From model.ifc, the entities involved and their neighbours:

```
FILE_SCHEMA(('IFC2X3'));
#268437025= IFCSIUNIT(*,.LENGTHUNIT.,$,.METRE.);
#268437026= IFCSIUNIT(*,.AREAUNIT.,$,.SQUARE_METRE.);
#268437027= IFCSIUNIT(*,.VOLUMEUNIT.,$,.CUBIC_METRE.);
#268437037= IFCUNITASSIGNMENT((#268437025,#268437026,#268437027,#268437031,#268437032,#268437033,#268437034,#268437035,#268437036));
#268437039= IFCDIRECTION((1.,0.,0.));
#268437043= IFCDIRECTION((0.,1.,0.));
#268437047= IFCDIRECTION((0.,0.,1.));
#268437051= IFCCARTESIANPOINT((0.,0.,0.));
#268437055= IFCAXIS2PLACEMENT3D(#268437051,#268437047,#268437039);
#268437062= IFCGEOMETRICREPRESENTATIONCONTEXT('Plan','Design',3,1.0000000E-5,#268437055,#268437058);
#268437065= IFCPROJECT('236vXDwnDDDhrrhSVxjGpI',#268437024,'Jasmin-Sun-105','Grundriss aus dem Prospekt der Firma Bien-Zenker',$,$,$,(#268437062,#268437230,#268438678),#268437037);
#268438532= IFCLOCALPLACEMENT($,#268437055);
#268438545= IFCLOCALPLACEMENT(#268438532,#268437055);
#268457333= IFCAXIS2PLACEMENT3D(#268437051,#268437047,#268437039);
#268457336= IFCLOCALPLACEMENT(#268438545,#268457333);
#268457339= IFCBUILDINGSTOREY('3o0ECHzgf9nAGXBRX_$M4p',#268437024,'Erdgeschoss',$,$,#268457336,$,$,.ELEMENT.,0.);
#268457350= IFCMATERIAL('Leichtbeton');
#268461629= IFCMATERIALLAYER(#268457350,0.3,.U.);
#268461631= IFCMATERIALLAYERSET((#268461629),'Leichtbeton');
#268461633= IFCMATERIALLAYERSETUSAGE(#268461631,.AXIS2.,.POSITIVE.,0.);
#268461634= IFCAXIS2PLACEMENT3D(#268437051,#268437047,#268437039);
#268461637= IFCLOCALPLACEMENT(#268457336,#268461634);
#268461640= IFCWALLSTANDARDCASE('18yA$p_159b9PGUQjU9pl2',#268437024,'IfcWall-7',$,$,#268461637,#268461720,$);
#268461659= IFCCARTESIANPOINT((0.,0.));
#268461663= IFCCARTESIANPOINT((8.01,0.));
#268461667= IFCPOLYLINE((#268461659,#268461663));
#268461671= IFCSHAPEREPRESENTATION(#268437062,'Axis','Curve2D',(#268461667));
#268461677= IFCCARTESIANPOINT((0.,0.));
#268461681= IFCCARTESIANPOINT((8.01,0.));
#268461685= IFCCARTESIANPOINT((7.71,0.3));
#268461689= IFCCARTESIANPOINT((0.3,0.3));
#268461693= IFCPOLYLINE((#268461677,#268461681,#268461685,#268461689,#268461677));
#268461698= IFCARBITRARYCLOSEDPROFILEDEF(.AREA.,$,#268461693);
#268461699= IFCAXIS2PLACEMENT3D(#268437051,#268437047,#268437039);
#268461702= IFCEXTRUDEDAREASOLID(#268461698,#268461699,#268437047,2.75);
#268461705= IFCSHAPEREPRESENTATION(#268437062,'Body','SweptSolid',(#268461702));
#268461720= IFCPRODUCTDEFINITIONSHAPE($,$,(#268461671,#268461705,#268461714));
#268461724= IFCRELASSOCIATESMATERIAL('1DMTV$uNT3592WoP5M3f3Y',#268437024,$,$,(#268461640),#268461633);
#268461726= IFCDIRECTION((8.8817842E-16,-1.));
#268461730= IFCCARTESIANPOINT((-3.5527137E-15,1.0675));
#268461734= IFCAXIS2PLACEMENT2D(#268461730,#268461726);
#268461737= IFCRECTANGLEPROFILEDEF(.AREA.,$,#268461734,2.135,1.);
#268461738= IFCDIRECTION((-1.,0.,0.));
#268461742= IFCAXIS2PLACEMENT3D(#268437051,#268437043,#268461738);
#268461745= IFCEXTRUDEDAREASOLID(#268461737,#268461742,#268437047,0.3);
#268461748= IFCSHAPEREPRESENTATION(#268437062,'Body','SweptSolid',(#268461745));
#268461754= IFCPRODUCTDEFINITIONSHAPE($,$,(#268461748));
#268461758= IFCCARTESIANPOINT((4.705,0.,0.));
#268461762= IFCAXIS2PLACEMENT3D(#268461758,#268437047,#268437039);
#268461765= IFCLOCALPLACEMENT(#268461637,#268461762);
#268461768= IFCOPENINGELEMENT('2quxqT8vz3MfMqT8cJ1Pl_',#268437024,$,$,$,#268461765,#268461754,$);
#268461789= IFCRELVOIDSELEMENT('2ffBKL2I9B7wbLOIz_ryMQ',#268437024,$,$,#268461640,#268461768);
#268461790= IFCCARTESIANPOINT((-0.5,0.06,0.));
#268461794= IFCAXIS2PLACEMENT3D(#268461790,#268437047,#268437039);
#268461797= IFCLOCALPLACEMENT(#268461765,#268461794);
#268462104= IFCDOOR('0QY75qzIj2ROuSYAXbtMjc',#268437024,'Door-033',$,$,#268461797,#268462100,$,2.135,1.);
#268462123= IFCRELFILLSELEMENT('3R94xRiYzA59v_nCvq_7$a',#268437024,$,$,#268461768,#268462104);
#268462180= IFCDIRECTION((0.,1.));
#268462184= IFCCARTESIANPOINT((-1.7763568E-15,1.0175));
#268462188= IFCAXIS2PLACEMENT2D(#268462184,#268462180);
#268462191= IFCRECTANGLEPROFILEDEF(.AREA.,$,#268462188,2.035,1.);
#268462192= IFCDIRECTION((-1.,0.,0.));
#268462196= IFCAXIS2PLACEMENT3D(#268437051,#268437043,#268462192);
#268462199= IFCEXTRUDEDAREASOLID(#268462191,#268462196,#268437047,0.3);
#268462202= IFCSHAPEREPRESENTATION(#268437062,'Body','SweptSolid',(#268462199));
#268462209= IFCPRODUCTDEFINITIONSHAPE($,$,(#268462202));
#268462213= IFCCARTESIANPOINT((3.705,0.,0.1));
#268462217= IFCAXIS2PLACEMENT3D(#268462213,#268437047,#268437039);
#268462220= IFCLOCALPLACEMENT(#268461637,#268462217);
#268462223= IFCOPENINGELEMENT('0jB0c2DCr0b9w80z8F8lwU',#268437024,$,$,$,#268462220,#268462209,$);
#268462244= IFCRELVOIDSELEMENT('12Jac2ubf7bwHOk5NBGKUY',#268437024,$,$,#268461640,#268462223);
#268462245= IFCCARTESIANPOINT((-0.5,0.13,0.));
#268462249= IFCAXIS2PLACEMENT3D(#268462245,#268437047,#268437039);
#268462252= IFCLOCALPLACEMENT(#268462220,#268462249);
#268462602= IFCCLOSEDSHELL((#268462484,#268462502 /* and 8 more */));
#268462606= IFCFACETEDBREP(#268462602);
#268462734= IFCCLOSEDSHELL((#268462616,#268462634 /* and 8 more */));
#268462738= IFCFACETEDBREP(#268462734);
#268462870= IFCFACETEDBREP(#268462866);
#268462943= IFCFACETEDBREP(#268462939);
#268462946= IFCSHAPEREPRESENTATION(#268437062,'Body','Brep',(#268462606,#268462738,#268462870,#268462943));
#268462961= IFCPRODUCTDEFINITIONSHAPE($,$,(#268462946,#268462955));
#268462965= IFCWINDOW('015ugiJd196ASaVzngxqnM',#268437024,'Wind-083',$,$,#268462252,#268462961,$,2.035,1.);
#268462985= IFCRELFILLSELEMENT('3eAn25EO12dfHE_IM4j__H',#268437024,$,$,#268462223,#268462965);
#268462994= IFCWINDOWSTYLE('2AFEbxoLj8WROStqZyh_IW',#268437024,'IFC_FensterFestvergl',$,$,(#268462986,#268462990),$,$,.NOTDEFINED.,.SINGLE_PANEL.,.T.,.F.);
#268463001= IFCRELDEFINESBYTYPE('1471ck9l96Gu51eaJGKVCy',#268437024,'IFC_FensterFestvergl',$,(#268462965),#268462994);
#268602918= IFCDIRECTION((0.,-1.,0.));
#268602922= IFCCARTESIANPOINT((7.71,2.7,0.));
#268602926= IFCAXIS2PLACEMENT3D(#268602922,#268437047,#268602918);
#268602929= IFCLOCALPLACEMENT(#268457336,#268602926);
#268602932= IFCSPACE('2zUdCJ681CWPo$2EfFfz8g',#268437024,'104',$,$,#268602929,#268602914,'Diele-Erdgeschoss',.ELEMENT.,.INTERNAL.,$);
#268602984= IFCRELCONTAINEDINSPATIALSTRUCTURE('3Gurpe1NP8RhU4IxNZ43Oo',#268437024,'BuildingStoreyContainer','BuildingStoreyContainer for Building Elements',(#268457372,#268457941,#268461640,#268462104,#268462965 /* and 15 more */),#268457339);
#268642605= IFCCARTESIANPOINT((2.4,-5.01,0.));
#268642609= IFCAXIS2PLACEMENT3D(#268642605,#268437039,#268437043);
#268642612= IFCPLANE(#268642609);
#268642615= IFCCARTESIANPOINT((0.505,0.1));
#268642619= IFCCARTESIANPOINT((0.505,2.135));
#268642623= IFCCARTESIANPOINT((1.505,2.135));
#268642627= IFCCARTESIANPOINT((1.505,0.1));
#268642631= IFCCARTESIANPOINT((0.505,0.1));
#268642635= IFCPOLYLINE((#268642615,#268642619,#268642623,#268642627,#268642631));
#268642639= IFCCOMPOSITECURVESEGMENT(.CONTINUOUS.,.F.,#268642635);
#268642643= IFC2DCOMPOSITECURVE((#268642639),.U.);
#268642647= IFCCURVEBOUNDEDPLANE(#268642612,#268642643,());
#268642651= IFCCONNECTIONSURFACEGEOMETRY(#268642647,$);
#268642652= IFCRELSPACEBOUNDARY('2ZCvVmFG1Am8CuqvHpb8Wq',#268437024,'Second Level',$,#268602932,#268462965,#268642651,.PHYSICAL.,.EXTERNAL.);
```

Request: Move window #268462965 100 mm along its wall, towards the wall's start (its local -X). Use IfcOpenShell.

```python
import numpy as np
import ifcopenshell
import ifcopenshell.api.geometry
import ifcopenshell.util.placement
import ifcopenshell.util.unit

model = ifcopenshell.open("model.ifc")
unit_scale = ifcopenshell.util.unit.calculate_unit_scale(model)

window = model.by_guid("015ugiJd196ASaVzngxqnM")
opening = window.FillsVoids[0].RelatingOpeningElement
wall = opening.VoidsElements[0].RelatingBuildingElement

wall_matrix = ifcopenshell.util.placement.get_local_placement(wall.ObjectPlacement)
shift = wall_matrix[:3, 0] * -0.1 / unit_scale
before = ifcopenshell.util.placement.get_local_placement(window.ObjectPlacement)[:3, 3].copy()

# The window is placed relative to its opening, so it follows when the opening moves.
matrix = ifcopenshell.util.placement.get_local_placement(opening.ObjectPlacement)
matrix[:3, 3] += shift
ifcopenshell.api.geometry.edit_object_placement(
    model, product=opening, matrix=matrix, is_si=False, should_transform_children=True
)

# Space boundary surfaces are stored in each space's coordinates; move them too.
for rel in window.ProvidesBoundaries:
    if not rel.ConnectionGeometry:
        continue
    surface = rel.ConnectionGeometry.SurfaceOnRelatingElement.BasisSurface
    space_matrix = ifcopenshell.util.placement.get_local_placement(rel.RelatingSpace.ObjectPlacement)
    point = np.array(surface.Position.Location.Coordinates) + space_matrix[:3, :3].T @ shift
    surface.Position = model.createIfcAxis2Placement3D(
        model.createIfcCartesianPoint(point.tolist()), surface.Position.Axis, surface.Position.RefDirection
    )

after = ifcopenshell.util.placement.get_local_placement(window.ObjectPlacement)[:3, 3]
print("window moved by", (after - before).round(3) + 0.0)

model.write("model_v2.ifc")
```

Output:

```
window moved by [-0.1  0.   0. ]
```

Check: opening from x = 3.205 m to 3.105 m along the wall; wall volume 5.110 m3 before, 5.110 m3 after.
